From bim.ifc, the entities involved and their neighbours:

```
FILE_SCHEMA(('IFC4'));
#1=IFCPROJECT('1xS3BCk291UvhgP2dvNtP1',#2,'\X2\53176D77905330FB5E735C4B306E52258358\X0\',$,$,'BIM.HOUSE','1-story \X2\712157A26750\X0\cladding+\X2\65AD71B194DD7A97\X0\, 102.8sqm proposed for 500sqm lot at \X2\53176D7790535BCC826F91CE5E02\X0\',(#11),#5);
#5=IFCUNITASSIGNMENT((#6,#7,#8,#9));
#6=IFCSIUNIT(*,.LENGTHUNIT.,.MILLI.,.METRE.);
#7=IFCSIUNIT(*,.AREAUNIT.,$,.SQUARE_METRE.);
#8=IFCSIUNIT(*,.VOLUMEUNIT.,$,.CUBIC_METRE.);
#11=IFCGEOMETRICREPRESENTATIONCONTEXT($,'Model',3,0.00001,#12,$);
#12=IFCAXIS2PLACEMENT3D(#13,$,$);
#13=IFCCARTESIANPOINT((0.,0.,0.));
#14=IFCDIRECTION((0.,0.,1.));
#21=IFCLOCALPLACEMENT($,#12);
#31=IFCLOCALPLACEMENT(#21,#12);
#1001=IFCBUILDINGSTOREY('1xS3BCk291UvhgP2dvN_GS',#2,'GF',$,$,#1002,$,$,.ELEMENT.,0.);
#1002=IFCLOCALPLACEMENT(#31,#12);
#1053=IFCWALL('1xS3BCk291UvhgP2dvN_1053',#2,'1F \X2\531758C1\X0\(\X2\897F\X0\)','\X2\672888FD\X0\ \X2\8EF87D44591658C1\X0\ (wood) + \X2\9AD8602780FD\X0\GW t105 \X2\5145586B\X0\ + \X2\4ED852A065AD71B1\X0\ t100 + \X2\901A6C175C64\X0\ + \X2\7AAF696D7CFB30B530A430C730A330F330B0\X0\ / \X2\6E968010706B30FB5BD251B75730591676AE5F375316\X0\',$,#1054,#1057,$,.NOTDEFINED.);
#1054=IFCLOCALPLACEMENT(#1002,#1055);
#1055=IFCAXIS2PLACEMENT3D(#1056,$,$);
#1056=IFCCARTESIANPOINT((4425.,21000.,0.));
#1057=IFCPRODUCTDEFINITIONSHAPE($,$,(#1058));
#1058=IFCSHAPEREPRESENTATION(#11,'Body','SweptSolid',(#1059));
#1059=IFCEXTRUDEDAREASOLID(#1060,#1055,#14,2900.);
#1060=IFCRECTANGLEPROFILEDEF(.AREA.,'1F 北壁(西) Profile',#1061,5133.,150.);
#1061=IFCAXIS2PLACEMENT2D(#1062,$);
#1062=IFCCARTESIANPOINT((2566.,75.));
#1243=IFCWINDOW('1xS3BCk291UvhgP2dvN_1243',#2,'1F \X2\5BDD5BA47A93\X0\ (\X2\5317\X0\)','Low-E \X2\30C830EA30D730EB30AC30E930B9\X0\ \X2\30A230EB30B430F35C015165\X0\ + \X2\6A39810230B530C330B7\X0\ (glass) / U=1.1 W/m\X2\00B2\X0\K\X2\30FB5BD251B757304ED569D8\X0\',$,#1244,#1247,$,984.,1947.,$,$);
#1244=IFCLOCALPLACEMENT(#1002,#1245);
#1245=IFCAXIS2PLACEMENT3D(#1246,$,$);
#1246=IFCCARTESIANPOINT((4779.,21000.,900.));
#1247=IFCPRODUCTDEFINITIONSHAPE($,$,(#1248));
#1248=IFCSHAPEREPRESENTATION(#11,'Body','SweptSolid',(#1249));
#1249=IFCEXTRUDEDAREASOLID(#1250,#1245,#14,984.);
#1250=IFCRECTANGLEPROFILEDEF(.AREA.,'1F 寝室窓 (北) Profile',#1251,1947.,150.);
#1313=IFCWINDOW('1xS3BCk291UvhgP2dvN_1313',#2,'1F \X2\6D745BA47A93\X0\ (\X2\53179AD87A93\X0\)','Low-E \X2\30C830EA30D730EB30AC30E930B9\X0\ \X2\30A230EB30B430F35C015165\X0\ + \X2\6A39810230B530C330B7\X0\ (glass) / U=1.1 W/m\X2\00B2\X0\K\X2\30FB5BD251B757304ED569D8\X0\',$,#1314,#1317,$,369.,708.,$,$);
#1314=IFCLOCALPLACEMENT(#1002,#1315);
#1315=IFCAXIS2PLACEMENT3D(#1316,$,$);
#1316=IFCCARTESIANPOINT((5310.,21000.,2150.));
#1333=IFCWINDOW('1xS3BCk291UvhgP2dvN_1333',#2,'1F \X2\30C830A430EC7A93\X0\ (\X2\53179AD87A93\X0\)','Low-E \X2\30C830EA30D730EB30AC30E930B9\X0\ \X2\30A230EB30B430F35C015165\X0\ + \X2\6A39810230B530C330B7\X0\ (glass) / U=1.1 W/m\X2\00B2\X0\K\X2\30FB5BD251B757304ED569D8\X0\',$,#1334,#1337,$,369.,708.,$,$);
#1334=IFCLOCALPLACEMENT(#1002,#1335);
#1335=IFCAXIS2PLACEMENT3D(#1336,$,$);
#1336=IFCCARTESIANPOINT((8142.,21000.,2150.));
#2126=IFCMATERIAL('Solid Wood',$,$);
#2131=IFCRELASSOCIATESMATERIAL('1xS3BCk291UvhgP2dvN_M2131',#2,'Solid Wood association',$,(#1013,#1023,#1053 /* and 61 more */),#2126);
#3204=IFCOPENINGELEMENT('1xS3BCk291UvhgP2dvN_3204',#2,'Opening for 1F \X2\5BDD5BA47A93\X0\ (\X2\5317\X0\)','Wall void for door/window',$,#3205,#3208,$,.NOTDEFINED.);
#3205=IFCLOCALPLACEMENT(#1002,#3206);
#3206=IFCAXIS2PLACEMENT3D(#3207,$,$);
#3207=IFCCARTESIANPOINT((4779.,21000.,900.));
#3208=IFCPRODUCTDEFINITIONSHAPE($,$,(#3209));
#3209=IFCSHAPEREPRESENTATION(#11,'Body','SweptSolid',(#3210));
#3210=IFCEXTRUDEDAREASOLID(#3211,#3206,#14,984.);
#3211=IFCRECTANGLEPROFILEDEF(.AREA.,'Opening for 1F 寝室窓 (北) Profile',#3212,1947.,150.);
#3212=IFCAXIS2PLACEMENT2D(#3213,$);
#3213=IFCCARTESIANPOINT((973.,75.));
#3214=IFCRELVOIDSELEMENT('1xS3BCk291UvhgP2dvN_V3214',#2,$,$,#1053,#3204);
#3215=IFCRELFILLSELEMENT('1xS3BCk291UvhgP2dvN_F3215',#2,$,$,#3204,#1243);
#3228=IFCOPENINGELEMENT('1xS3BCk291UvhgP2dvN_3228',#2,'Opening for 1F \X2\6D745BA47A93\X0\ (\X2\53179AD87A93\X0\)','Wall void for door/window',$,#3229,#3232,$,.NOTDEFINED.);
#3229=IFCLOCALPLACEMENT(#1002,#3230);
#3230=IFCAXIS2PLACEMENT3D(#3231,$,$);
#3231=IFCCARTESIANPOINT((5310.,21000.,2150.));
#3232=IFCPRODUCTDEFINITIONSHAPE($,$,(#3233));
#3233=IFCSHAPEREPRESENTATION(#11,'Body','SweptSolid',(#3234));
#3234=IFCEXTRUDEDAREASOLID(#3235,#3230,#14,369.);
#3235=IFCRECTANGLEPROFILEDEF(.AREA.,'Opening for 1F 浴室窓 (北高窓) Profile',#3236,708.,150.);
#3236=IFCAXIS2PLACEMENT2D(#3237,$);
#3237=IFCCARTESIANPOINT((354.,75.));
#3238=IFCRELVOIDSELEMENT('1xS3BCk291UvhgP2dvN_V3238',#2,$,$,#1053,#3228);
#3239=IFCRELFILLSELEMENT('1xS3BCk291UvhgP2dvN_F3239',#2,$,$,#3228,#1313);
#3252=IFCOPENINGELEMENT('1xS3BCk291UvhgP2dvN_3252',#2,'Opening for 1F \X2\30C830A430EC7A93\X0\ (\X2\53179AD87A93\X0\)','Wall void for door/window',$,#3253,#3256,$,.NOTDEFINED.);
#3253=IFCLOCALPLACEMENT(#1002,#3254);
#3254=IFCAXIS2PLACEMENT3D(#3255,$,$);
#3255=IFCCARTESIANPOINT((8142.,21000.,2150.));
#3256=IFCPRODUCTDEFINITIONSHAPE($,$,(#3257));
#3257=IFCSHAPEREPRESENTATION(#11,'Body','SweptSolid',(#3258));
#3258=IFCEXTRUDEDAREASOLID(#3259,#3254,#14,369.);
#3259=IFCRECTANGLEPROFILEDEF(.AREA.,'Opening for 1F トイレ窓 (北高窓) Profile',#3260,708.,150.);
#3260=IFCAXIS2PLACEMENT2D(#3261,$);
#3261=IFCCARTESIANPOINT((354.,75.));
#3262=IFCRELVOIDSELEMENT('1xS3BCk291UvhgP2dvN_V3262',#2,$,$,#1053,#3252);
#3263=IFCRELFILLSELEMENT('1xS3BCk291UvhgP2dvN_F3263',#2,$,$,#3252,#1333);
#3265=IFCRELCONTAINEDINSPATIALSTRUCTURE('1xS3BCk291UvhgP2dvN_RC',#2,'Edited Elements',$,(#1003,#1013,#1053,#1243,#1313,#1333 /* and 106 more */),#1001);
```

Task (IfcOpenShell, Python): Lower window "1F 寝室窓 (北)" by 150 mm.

```python
import numpy as np
import ifcopenshell
import ifcopenshell.api.geometry
import ifcopenshell.util.placement
import ifcopenshell.util.unit

model = ifcopenshell.open("bim.ifc")
unit_scale = ifcopenshell.util.unit.calculate_unit_scale(model)

window = model.by_guid("1xS3BCk291UvhgP2dvN_1243")
opening = window.FillsVoids[0].RelatingOpeningElement
dz = -150.0

shift = np.array([0.0, 0.0, dz])
# The window is not placed relative to its opening, so move both.
for product in (opening, window):
    matrix = ifcopenshell.util.placement.get_local_placement(product.ObjectPlacement)
    matrix[:3, 3] += shift
    ifcopenshell.api.geometry.edit_object_placement(model, product=product, matrix=matrix, is_si=False)

print(f"moved by {dz * unit_scale:+.3f} m")

model.write("bim_edited.ifc")
```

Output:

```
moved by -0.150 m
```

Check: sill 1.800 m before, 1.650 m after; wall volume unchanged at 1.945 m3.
